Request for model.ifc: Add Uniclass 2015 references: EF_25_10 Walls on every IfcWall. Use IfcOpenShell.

First a look at what the model holds.

```python
import ifcopenshell

model = ifcopenshell.open("model.ifc")
print(model.schema)
print("classifications:", [c.Name for c in model.by_type("IfcClassification")])
for ifc_class in ("IfcDoor", "IfcRoof", "IfcStair", "IfcWall", "IfcWindow"):
    print(ifc_class, len(model.by_type(ifc_class)))
```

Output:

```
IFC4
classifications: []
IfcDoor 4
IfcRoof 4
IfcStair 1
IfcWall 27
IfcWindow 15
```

```python
import ifcopenshell
import ifcopenshell.api.classification

model = ifcopenshell.open("model.ifc")

system = ifcopenshell.api.classification.add_classification(model, classification="Uniclass 2015")

codes = {
    "IfcWall": ("EF_25_10", "Walls"),
}
for ifc_class, (code, name) in codes.items():
    products = model.by_type(ifc_class)
    ifcopenshell.api.classification.add_reference(
        model, products=products, classification=system, identification=code, name=name
    )
    print(code, len(products))

model.write("model_updated.ifc")
```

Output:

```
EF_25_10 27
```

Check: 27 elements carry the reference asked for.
